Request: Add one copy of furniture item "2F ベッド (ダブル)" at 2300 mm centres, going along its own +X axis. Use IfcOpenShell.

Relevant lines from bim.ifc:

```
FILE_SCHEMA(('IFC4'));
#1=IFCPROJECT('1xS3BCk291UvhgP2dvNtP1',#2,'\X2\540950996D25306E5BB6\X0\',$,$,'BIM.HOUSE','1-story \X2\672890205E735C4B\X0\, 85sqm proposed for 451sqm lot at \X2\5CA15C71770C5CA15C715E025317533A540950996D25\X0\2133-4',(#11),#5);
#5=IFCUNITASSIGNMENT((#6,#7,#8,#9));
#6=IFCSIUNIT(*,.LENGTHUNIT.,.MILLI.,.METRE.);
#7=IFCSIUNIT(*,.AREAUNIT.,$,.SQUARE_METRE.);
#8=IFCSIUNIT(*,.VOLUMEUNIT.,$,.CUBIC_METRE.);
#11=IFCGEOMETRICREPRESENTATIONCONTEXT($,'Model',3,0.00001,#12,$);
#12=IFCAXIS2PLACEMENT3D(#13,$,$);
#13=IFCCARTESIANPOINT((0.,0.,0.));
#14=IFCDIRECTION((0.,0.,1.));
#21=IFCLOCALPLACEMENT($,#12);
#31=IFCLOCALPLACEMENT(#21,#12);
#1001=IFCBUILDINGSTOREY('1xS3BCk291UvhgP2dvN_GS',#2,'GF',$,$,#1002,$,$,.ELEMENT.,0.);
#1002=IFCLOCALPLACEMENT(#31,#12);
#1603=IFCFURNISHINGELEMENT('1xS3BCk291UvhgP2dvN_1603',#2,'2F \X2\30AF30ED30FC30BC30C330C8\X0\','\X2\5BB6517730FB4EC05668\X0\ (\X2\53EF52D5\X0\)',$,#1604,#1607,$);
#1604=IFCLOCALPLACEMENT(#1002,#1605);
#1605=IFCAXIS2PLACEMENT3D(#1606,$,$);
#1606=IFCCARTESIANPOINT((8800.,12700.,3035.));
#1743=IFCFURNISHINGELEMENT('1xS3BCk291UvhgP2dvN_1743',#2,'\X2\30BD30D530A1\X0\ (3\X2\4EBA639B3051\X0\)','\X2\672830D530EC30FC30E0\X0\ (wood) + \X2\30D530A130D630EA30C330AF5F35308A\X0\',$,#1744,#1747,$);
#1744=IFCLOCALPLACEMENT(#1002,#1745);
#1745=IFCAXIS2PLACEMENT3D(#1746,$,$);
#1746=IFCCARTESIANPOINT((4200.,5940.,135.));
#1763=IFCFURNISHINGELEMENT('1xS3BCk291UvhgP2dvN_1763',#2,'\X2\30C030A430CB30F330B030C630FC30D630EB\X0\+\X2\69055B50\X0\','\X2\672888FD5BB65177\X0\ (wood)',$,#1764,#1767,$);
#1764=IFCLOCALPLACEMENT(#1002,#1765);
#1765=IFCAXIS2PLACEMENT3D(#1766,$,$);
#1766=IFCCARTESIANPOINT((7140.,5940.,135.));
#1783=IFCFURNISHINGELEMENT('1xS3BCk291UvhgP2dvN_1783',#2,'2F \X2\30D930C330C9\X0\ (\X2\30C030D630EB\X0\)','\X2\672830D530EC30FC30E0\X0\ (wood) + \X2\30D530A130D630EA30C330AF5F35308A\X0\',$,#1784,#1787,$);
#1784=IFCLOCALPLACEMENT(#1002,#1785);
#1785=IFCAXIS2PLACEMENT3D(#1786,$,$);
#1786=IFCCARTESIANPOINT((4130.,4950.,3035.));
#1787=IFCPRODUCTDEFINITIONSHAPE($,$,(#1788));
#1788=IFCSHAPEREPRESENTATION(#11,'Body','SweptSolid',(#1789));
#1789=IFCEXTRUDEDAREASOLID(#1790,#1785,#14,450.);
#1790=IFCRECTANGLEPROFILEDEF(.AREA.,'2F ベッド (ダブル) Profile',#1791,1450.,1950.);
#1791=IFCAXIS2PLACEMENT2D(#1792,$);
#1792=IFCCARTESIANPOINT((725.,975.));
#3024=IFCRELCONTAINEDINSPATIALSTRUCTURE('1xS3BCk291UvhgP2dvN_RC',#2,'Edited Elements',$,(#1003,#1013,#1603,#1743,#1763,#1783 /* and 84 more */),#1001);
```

```python
import ifcopenshell
import ifcopenshell.api.geometry
import ifcopenshell.api.root
import ifcopenshell.util.element
import ifcopenshell.util.placement

model = ifcopenshell.open("bim.ifc")


def reuse_history(source, copy):
    """copy_class also copies each property set's owner history, people and application; keep the originals."""
    for rel in copy.IsDefinedBy:
        if rel.is_a("IfcRelDefinesByProperties") and (history := rel.RelatingPropertyDefinition.OwnerHistory):
            rel.RelatingPropertyDefinition.OwnerHistory = source.OwnerHistory
            ifcopenshell.util.element.remove_deep2(model, history)


source = model.by_guid("1xS3BCk291UvhgP2dvN_1783")
base = ifcopenshell.util.placement.get_local_placement(source.ObjectPlacement)
step = base[:3, 0] * 2300.0

for i in range(1, 2):
    copy = ifcopenshell.api.root.copy_class(model, product=source)
    copy.Representation = ifcopenshell.util.element.copy_deep(
        model, source.Representation, exclude=["IfcGeometricRepresentationContext", "IfcRepresentationMap"]
    )
    reuse_history(source, copy)
    matrix = base.copy()
    matrix[:3, 3] += i * step
    print("added at", matrix[:3, 3].round(3) + 0.0)
    ifcopenshell.api.geometry.edit_object_placement(model, product=copy, matrix=matrix, is_si=False)

model.write("bim_edited.ifc")
```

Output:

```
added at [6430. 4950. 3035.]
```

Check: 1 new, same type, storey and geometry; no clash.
